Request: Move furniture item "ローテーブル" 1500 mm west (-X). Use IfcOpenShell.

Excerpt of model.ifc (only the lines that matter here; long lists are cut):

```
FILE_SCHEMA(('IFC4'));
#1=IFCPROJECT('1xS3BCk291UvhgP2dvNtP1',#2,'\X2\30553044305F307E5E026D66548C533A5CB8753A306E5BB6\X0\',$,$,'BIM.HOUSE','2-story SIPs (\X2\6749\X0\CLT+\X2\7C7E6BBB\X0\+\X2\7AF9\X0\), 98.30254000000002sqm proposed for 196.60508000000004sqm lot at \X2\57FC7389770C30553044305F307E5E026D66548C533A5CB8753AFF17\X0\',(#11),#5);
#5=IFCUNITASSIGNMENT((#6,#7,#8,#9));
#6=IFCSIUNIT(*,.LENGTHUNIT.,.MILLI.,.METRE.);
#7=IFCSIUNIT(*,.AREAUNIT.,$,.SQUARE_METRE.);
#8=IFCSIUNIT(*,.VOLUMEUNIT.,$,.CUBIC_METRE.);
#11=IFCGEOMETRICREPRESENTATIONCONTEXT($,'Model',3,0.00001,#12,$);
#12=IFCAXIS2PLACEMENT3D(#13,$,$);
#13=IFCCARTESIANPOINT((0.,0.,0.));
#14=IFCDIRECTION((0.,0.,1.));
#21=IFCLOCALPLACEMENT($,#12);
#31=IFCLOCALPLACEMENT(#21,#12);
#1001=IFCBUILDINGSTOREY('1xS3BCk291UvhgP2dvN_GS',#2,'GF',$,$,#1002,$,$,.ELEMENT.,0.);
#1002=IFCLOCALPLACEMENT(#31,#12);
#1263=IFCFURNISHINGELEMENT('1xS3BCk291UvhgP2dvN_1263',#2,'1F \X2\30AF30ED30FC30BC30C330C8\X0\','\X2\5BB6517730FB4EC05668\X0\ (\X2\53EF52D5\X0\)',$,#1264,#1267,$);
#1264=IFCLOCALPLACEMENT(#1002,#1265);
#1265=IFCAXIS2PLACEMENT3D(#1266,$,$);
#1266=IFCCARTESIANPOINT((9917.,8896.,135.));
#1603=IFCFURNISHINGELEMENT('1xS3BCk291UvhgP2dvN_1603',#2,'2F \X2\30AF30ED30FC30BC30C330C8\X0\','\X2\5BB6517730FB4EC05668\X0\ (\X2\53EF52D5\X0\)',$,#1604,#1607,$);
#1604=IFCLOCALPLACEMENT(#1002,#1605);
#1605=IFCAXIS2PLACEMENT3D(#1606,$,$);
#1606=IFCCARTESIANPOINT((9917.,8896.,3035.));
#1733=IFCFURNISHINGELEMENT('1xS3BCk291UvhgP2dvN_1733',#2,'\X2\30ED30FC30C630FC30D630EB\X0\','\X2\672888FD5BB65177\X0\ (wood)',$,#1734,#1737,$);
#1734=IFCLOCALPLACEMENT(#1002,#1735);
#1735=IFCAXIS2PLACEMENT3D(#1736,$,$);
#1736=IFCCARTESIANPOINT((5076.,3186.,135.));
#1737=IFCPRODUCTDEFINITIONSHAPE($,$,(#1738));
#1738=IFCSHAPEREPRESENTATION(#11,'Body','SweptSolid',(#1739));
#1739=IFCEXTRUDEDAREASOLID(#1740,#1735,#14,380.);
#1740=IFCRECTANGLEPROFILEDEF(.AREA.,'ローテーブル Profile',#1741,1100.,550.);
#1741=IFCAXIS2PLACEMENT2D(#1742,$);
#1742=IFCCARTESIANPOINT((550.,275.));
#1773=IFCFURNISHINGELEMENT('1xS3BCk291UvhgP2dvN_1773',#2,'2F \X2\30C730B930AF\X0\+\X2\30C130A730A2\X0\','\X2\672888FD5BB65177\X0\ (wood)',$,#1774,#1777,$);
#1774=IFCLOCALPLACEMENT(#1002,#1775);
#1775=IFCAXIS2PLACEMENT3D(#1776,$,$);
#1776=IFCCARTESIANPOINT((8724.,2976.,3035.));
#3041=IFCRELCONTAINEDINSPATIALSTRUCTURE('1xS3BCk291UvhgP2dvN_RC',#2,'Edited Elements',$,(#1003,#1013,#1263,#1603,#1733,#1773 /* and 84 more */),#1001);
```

```python
import ifcopenshell
import ifcopenshell.api.geometry
import ifcopenshell.util.placement
import ifcopenshell.util.unit

model = ifcopenshell.open("model.ifc")
unit_scale = ifcopenshell.util.unit.calculate_unit_scale(model)

item = model.by_id(1733)
matrix = ifcopenshell.util.placement.get_local_placement(item.ObjectPlacement)
matrix[0, 3] -= 1.5 / unit_scale
ifcopenshell.api.geometry.edit_object_placement(model, product=item, matrix=matrix, is_si=False)

print(ifcopenshell.util.placement.get_local_placement(item.ObjectPlacement).round(3) + 0.0)

model.write("model_rev.ifc")
```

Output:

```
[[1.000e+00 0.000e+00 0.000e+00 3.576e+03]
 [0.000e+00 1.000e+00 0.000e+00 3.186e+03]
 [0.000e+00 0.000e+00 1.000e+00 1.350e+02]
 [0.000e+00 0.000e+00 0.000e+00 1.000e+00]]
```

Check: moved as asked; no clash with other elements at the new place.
